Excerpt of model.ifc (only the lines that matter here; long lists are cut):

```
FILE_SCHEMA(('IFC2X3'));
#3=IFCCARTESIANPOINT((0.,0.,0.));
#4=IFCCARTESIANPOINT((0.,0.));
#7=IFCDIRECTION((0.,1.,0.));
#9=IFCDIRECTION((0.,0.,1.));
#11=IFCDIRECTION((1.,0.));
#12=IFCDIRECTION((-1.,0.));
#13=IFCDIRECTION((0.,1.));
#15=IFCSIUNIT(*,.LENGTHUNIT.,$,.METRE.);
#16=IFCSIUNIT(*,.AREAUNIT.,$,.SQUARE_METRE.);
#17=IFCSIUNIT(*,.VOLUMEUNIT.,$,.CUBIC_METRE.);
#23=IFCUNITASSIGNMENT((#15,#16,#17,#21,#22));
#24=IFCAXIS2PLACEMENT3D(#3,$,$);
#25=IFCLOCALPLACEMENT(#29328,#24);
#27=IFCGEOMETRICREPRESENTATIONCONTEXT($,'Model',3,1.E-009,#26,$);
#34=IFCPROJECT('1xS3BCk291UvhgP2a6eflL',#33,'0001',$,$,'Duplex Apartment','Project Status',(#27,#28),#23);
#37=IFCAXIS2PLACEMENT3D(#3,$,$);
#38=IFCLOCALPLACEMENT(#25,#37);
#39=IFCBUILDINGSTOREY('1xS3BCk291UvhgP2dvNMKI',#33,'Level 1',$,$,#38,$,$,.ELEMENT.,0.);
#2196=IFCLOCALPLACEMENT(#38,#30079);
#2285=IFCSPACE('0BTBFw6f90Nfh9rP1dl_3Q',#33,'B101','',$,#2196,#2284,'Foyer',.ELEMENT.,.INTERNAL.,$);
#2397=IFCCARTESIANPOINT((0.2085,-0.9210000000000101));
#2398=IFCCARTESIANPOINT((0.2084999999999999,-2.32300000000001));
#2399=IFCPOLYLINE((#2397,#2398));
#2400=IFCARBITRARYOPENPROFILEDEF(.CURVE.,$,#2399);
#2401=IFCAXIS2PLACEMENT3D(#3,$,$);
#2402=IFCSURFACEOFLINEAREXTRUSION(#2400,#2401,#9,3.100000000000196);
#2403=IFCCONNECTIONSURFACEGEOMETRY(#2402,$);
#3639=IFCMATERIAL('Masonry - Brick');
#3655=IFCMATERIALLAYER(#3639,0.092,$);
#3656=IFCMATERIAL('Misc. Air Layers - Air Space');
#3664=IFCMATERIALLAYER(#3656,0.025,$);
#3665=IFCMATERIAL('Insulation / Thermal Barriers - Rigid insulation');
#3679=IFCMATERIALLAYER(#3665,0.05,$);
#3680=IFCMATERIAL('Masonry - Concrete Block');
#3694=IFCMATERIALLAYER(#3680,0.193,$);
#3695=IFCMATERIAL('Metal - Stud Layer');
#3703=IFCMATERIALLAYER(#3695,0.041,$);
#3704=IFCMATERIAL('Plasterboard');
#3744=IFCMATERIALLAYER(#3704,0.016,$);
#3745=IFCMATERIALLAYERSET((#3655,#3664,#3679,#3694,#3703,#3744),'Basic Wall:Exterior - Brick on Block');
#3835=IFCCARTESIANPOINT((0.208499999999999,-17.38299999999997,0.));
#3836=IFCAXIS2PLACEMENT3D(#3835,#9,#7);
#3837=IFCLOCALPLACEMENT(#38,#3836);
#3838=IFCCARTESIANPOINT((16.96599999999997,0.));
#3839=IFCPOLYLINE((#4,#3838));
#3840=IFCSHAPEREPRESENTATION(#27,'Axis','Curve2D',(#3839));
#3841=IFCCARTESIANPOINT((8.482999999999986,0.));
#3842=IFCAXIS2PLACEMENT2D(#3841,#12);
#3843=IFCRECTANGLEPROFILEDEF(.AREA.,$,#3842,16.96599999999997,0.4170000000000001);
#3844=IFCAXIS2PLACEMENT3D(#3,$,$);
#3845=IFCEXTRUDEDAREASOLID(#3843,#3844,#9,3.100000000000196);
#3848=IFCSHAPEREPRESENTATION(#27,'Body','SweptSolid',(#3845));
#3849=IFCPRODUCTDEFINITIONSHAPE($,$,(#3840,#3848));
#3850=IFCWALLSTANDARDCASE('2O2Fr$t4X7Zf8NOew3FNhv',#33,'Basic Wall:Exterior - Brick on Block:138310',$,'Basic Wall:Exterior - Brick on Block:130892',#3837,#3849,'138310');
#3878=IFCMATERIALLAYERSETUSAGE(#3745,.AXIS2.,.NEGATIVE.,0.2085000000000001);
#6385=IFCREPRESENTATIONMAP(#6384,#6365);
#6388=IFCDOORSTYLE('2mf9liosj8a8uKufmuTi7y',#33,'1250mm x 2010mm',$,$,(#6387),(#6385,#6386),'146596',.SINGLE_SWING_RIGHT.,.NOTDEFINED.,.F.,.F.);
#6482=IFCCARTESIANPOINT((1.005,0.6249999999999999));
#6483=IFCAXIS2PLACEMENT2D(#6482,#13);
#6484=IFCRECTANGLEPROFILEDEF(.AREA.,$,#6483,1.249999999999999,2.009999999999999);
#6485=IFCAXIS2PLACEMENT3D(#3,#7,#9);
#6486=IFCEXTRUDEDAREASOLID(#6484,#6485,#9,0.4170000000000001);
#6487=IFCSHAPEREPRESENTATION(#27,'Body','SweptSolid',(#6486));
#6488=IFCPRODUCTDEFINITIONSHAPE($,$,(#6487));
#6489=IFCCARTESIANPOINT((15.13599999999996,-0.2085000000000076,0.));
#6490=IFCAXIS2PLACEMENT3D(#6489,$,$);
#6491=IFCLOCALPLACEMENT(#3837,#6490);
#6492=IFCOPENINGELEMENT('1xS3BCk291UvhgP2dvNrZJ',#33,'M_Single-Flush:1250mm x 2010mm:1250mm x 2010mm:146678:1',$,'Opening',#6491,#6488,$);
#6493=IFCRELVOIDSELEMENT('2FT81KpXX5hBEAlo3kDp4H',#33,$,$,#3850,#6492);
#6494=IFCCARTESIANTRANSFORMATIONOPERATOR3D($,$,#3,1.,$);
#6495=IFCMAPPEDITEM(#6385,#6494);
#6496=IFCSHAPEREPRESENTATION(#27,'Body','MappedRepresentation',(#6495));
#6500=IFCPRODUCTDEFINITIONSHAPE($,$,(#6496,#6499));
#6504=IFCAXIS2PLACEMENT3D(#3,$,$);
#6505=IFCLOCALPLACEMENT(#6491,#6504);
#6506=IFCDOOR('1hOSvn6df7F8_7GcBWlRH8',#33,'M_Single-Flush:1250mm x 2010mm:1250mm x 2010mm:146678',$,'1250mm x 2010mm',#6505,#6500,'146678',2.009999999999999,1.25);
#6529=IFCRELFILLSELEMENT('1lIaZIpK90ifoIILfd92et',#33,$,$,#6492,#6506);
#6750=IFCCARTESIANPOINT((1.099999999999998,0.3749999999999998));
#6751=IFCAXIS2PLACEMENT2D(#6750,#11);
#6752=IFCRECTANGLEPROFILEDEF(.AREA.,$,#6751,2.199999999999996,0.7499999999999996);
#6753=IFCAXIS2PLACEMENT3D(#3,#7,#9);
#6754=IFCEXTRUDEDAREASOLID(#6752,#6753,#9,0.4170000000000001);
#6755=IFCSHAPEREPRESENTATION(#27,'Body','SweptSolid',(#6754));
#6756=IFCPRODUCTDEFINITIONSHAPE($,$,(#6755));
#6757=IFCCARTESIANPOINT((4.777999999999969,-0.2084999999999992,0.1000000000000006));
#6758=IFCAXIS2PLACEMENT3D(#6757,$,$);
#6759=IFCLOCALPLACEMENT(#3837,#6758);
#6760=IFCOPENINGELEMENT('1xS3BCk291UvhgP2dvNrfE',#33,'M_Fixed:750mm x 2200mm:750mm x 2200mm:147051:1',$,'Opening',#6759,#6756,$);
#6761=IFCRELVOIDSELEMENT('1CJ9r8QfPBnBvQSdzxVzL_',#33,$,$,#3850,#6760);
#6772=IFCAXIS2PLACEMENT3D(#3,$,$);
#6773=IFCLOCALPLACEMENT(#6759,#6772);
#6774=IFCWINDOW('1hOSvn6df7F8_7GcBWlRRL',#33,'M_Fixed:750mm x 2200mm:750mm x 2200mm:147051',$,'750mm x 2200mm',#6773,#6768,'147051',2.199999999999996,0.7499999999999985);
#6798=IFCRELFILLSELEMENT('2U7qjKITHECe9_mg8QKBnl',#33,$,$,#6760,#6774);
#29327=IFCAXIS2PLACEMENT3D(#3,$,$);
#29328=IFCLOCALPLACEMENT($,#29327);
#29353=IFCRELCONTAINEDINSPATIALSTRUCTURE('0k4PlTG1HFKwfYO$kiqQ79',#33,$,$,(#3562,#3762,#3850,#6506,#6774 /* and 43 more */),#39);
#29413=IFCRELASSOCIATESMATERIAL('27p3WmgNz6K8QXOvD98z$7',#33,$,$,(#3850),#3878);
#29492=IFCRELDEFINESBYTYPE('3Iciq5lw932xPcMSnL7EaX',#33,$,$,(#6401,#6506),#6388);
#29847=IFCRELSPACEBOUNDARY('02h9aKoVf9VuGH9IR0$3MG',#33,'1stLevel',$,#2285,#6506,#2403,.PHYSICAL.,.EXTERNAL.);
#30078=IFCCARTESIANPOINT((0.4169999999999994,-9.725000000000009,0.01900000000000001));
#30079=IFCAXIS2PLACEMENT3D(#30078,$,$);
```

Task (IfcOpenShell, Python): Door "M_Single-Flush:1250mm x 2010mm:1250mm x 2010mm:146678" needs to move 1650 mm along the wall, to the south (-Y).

```python
import numpy as np
import ifcopenshell
import ifcopenshell.api.geometry
import ifcopenshell.util.placement
import ifcopenshell.util.unit

model = ifcopenshell.open("model.ifc")
unit_scale = ifcopenshell.util.unit.calculate_unit_scale(model)

door = model.by_guid("1hOSvn6df7F8_7GcBWlRH8")
opening = door.FillsVoids[0].RelatingOpeningElement
wall = opening.VoidsElements[0].RelatingBuildingElement

wall_matrix = ifcopenshell.util.placement.get_local_placement(wall.ObjectPlacement)
shift = wall_matrix[:3, 0] * -1.65 / unit_scale
before = ifcopenshell.util.placement.get_local_placement(door.ObjectPlacement)[:3, 3].copy()

# The door is placed relative to its opening, so it follows when the opening moves.
matrix = ifcopenshell.util.placement.get_local_placement(opening.ObjectPlacement)
matrix[:3, 3] += shift
ifcopenshell.api.geometry.edit_object_placement(
    model, product=opening, matrix=matrix, is_si=False, should_transform_children=True
)

# Space boundary surfaces are stored in each space's coordinates; move them too.
for rel in door.ProvidesBoundaries:
    if not rel.ConnectionGeometry:
        continue
    surface = rel.ConnectionGeometry.SurfaceOnRelatingElement
    space_matrix = ifcopenshell.util.placement.get_local_placement(rel.RelatingSpace.ObjectPlacement)
    point = np.array(surface.Position.Location.Coordinates) + space_matrix[:3, :3].T @ shift
    surface.Position = model.createIfcAxis2Placement3D(
        model.createIfcCartesianPoint(point.tolist()), surface.Position.Axis, surface.Position.RefDirection
    )

after = ifcopenshell.util.placement.get_local_placement(door.ObjectPlacement)[:3, 3]
print("door moved by", (after - before).round(3) + 0.0)

model.write("model-out.ifc")
```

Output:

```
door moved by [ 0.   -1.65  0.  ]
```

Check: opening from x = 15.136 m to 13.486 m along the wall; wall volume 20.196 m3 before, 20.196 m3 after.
